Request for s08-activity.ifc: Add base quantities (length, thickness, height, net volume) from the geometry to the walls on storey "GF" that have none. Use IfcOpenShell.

First a look at what the model holds.

```python
import ifcopenshell
import ifcopenshell.util.element
import ifcopenshell.util.unit

model = ifcopenshell.open("s08-activity.ifc")
print(model.schema)
for unit_type in ("LENGTHUNIT", "AREAUNIT", "VOLUMEUNIT"):
    print(unit_type, ifcopenshell.util.unit.calculate_unit_scale(model, unit_type))
storey = next(s for s in model.by_type("IfcBuildingStorey") if s.Name == "GF")
walls = [e for e in ifcopenshell.util.element.get_decomposition(storey) if e.is_a("IfcWall")]
for e in sorted(walls, key=lambda e: e.id()):
    print(e.id(), e.is_a(), e.Name, list(ifcopenshell.util.element.get_psets(e, qtos_only=True)), sep=" | ")
```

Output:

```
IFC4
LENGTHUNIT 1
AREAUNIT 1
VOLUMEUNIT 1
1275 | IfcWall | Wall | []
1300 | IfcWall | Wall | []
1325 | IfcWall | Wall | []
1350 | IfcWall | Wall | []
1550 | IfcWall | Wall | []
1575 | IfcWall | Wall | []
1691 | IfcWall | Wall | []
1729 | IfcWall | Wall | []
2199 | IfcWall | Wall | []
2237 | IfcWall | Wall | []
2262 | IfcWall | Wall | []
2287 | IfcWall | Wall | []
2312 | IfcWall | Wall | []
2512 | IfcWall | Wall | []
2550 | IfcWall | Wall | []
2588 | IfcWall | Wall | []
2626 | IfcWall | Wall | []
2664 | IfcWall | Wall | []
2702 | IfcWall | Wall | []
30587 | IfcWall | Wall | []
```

```python
import ifcopenshell
import ifcopenshell.api.pset
import ifcopenshell.geom
import ifcopenshell.util.element
import ifcopenshell.util.shape
import ifcopenshell.util.unit

model = ifcopenshell.open("s08-activity.ifc")
unit_scale = ifcopenshell.util.unit.calculate_unit_scale(model)
volume_scale = ifcopenshell.util.unit.calculate_unit_scale(model, "VOLUMEUNIT")
settings = ifcopenshell.geom.settings()

storey = next(s for s in model.by_type("IfcBuildingStorey") if s.Name == "GF")
walls = [e for e in ifcopenshell.util.element.get_decomposition(storey) if e.is_a("IfcWall")]

for e in sorted(walls, key=lambda e: e.id()):
    if ifcopenshell.util.element.get_psets(e, qtos_only=True, should_inherit=False):
        continue
    # Geometry comes back in metres, in the element's own axes.
    shape = ifcopenshell.geom.create_shape(settings, e)
    values = {
        "Length": ifcopenshell.util.shape.get_x(shape.geometry) / unit_scale,
        "Width": ifcopenshell.util.shape.get_y(shape.geometry) / unit_scale,
        "Height": ifcopenshell.util.shape.get_z(shape.geometry) / unit_scale,
        "NetVolume": ifcopenshell.util.shape.get_volume(shape.geometry) / volume_scale,
    }
    qto = ifcopenshell.api.pset.add_qto(model, product=e, name="Qto_WallBaseQuantities")
    ifcopenshell.api.pset.edit_qto(model, qto=qto, properties=values)
    print(e.id(), {k: round(v, 3) for k, v in values.items()})

model.write("s08-activity_edited.ifc")
```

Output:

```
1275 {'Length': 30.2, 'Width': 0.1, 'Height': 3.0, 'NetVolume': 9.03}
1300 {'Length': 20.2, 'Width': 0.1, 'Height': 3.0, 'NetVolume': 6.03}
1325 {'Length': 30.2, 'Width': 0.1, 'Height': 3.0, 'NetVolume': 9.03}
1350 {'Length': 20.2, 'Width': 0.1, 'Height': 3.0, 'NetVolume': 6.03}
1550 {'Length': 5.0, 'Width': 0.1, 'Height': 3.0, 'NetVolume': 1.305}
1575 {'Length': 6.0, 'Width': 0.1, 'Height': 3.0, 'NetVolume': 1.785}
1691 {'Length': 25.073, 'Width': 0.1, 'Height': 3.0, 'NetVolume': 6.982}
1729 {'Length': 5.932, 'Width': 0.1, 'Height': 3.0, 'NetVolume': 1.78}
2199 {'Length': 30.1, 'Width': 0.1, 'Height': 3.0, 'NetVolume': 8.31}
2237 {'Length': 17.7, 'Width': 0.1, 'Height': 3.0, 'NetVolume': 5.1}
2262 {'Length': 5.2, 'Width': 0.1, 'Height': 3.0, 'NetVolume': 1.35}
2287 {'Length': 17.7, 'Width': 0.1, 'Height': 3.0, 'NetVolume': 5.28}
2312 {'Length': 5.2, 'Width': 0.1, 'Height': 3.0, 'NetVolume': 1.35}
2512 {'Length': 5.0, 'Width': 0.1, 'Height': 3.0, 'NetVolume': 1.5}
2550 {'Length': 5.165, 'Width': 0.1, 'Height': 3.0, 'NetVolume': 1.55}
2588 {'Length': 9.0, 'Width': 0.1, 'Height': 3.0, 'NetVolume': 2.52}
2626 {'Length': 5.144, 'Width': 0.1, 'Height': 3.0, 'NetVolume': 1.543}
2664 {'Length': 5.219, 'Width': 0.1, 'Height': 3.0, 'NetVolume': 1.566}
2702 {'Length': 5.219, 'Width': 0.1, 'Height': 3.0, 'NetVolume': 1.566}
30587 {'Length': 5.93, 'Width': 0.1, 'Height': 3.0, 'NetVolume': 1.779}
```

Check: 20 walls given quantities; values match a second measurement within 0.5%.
